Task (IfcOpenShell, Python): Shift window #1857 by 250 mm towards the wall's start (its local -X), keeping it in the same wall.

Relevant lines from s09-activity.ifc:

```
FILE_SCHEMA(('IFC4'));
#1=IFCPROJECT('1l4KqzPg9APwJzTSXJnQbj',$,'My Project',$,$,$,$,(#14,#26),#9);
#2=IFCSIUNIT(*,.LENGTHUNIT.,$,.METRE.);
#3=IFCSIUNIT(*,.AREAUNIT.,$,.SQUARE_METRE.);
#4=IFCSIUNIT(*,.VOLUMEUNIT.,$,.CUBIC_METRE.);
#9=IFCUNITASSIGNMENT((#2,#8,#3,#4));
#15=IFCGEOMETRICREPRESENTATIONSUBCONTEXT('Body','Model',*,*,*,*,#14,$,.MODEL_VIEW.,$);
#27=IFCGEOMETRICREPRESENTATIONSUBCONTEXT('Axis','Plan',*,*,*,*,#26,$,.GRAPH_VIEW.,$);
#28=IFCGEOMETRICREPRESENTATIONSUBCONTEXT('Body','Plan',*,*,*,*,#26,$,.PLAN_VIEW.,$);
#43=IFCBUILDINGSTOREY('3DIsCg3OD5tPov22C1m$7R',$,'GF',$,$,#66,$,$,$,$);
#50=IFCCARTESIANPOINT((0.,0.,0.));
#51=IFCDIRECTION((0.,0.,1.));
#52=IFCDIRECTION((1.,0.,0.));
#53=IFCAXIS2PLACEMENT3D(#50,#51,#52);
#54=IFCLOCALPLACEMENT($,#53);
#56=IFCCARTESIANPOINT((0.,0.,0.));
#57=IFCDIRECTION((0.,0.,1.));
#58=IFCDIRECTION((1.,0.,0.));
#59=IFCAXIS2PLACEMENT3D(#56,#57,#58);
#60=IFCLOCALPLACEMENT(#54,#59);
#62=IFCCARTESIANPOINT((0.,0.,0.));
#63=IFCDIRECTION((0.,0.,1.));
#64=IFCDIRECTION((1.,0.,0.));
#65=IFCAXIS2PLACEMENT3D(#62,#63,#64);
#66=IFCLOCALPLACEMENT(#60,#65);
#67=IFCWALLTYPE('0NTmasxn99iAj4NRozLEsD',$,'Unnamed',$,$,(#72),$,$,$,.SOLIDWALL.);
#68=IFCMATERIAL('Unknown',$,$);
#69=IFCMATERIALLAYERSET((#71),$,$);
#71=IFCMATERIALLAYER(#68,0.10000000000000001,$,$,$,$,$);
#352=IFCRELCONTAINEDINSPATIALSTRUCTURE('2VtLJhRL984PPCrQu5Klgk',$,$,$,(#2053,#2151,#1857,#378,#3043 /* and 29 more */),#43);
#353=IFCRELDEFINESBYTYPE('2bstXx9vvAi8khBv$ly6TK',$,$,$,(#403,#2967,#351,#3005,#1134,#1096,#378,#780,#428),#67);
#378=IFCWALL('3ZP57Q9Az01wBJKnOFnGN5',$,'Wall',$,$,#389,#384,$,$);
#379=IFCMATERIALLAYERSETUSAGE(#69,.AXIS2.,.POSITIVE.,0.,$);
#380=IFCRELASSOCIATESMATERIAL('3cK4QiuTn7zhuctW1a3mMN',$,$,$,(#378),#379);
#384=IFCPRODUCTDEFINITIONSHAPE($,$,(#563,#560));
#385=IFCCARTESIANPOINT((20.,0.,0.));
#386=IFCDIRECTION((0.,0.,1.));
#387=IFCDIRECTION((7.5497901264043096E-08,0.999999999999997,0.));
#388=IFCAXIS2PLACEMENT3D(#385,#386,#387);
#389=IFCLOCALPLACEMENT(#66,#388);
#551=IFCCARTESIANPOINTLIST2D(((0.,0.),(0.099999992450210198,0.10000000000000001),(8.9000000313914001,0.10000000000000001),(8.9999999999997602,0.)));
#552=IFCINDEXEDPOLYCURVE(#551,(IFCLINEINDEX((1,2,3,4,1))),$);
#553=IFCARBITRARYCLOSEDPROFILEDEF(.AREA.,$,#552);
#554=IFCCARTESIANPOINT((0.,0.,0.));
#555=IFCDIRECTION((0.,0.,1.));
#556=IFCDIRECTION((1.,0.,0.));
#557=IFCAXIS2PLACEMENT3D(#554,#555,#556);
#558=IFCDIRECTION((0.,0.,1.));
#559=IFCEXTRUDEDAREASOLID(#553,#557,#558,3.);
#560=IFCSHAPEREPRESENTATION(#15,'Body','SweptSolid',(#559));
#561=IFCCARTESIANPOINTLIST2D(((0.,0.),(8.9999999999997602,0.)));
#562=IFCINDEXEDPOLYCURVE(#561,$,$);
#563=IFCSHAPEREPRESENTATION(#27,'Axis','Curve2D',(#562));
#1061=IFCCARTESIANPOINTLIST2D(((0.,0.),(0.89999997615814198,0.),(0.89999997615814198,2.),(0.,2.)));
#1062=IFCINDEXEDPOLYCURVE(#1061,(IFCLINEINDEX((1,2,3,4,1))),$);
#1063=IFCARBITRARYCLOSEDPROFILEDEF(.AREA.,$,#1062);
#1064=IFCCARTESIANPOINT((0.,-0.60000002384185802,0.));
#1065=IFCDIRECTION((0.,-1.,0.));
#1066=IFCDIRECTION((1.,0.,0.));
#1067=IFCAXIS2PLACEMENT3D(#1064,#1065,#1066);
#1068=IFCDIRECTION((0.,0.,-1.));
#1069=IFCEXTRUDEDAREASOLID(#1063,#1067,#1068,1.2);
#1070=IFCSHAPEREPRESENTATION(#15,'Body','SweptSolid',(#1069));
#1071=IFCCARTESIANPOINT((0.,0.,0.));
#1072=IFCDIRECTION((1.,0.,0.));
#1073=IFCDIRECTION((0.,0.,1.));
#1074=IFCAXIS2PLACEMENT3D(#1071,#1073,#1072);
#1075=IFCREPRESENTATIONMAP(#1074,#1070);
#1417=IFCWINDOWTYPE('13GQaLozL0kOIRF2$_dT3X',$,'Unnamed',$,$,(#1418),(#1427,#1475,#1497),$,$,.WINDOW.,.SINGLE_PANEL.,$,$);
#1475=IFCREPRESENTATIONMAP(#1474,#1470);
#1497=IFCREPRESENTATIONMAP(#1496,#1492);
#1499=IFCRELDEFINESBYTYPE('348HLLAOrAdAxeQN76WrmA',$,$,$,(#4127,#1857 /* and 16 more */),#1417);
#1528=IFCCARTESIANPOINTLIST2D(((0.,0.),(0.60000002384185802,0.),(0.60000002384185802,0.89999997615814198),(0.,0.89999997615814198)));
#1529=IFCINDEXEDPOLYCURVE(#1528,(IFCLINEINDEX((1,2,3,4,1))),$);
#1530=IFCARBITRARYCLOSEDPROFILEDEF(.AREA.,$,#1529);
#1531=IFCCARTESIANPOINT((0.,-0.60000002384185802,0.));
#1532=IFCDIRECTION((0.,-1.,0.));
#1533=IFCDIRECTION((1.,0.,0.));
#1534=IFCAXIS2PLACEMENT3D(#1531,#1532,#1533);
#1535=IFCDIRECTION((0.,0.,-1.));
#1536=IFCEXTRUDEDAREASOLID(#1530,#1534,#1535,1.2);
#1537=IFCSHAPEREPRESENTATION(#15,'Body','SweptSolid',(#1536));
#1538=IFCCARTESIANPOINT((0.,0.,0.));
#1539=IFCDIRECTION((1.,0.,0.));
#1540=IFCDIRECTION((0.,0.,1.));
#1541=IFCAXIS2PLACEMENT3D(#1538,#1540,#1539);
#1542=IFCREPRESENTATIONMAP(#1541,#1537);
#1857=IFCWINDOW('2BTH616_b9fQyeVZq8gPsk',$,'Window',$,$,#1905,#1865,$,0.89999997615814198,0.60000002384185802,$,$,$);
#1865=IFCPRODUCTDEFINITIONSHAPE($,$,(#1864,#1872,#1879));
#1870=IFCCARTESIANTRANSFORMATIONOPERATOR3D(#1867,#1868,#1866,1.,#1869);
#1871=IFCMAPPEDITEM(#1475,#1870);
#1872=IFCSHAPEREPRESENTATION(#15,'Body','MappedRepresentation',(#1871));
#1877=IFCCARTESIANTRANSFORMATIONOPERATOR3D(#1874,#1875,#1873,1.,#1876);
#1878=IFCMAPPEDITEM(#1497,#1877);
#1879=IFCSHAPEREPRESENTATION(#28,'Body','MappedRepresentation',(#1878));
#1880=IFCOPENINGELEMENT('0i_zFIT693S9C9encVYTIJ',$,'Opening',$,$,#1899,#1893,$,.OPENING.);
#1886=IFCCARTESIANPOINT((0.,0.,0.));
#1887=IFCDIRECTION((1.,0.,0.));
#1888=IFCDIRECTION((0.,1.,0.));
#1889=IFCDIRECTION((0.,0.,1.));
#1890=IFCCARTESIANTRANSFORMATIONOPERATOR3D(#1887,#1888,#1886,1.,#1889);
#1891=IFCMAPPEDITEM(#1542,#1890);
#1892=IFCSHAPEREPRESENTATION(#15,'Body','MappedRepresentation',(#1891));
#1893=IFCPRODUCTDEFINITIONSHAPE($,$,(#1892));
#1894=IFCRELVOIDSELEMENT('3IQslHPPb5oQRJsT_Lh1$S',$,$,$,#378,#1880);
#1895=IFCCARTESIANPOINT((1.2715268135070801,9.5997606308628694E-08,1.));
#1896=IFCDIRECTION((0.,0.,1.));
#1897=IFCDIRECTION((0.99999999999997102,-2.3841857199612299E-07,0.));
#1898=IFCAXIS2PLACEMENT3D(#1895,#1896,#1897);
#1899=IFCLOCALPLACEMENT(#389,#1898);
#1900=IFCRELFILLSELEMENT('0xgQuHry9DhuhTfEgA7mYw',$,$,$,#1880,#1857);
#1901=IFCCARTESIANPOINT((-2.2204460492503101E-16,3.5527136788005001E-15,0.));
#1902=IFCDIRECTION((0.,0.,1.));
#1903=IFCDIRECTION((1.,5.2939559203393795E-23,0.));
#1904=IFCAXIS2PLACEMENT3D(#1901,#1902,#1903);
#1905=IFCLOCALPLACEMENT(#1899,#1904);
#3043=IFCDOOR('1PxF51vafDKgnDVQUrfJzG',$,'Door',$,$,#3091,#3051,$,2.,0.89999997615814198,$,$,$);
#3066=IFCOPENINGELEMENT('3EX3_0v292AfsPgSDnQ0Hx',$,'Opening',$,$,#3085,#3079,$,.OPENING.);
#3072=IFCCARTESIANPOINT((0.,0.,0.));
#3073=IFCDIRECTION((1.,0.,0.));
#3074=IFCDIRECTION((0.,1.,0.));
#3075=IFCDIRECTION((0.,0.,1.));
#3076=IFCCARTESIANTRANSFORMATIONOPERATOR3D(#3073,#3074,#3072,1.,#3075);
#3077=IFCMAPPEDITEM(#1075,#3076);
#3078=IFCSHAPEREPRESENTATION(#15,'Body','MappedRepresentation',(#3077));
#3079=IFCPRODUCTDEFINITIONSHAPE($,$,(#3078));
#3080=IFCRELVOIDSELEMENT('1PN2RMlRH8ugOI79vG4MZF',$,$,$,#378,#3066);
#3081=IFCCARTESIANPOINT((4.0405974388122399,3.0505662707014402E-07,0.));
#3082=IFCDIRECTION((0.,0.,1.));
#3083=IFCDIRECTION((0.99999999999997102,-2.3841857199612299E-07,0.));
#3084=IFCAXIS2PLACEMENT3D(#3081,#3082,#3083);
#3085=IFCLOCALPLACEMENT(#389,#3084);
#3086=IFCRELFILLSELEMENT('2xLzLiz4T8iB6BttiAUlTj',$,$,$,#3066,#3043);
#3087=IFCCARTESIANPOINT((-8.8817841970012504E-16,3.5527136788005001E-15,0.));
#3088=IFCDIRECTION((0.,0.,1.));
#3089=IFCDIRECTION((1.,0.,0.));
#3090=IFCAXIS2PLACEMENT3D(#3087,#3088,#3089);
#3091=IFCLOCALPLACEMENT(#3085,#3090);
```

```python
import ifcopenshell
import ifcopenshell.api.geometry
import ifcopenshell.util.placement

model = ifcopenshell.open("s09-activity.ifc")

window = model.by_id(1857)
opening = window.FillsVoids[0].RelatingOpeningElement
wall = opening.VoidsElements[0].RelatingBuildingElement

wall_matrix = ifcopenshell.util.placement.get_local_placement(wall.ObjectPlacement)
shift = wall_matrix[:3, 0] * -0.25
before = ifcopenshell.util.placement.get_local_placement(window.ObjectPlacement)[:3, 3].copy()

# The window is placed relative to its opening, so it follows when the opening moves.
matrix = ifcopenshell.util.placement.get_local_placement(opening.ObjectPlacement)
matrix[:3, 3] += shift
ifcopenshell.api.geometry.edit_object_placement(
    model, product=opening, matrix=matrix, is_si=False, should_transform_children=True
)

after = ifcopenshell.util.placement.get_local_placement(window.ObjectPlacement)[:3, 3]
print("window moved by", (after - before).round(3) + 0.0)

model.write("s09-activity_edited.ifc")
```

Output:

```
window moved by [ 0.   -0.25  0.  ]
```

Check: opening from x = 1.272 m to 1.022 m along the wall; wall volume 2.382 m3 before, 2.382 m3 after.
